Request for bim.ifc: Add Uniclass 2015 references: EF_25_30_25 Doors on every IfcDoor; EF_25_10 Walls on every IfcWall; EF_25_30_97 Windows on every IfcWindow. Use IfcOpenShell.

First a look at what the model holds.

```python
import ifcopenshell

model = ifcopenshell.open("bim.ifc")
print(model.schema)
print("classifications:", [c.Name for c in model.by_type("IfcClassification")])
for ifc_class in ("IfcDoor", "IfcRoof", "IfcStair", "IfcWall", "IfcWindow"):
    print(ifc_class, len(model.by_type(ifc_class)))
```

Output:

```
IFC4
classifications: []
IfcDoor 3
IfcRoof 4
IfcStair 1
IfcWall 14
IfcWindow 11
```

```python
import ifcopenshell
import ifcopenshell.api.classification

model = ifcopenshell.open("bim.ifc")

system = ifcopenshell.api.classification.add_classification(model, classification="Uniclass 2015")

codes = {
    "IfcDoor": ("EF_25_30_25", "Doors"),
    "IfcWall": ("EF_25_10", "Walls"),
    "IfcWindow": ("EF_25_30_97", "Windows"),
}
for ifc_class, (code, name) in codes.items():
    products = model.by_type(ifc_class)
    ifcopenshell.api.classification.add_reference(
        model, products=products, classification=system, identification=code, name=name
    )
    print(code, len(products))

model.write("bim-out.ifc")
```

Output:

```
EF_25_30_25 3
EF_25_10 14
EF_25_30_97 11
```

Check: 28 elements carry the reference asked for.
